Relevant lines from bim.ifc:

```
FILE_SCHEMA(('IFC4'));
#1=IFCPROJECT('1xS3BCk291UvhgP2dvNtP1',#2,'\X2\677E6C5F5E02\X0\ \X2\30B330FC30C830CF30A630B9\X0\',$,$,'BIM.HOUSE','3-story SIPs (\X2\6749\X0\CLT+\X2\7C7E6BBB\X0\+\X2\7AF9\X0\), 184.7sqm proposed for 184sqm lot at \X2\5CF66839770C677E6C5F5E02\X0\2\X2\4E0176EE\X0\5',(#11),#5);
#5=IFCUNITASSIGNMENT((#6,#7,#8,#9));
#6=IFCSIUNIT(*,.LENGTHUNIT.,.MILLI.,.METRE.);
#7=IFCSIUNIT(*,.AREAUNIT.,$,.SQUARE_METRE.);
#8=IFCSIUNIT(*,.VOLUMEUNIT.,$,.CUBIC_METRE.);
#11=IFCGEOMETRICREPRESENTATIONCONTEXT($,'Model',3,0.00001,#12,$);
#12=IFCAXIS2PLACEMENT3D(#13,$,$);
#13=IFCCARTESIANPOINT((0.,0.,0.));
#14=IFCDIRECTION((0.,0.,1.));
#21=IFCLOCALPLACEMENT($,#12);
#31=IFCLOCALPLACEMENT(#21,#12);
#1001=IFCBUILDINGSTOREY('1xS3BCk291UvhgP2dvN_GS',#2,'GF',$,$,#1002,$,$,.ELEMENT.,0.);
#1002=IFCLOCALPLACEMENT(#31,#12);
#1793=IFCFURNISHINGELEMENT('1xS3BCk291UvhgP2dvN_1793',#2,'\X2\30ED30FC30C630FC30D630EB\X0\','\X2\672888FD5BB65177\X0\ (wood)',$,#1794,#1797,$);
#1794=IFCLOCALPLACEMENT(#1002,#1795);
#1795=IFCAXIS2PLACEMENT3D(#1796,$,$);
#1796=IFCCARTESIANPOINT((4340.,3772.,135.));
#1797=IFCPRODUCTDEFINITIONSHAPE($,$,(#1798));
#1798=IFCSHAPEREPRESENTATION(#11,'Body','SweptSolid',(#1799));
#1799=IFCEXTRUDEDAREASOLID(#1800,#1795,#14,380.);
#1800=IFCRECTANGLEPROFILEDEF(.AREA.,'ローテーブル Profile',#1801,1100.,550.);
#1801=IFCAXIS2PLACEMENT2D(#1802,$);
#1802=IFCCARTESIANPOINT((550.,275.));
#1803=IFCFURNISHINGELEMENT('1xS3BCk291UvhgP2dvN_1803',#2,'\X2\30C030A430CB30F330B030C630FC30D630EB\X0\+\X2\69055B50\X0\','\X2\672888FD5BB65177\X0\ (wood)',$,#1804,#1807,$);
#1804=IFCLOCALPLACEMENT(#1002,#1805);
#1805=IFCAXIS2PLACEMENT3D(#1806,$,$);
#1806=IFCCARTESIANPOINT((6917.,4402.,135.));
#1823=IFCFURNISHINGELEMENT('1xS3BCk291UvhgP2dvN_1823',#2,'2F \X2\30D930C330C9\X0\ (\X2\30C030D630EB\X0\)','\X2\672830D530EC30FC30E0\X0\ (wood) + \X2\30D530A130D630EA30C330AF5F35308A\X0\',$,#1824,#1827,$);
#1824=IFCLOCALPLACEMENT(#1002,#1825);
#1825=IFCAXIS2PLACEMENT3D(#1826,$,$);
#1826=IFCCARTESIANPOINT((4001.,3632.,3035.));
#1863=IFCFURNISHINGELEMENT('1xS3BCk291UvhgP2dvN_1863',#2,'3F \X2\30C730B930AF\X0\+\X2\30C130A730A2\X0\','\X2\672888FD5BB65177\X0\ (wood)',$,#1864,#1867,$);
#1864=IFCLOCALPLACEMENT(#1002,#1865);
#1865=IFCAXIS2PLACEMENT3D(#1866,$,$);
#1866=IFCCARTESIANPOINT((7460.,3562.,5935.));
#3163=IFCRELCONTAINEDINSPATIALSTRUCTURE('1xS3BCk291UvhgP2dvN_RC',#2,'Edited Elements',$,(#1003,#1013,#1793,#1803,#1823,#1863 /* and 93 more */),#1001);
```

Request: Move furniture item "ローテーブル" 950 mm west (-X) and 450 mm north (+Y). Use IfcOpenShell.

```python
import ifcopenshell
import ifcopenshell.api.geometry
import ifcopenshell.util.placement
import ifcopenshell.util.unit

model = ifcopenshell.open("bim.ifc")
unit_scale = ifcopenshell.util.unit.calculate_unit_scale(model)

item = model.by_guid("1xS3BCk291UvhgP2dvN_1793")
matrix = ifcopenshell.util.placement.get_local_placement(item.ObjectPlacement)
matrix[0, 3] -= 0.95 / unit_scale
matrix[1, 3] += 0.45 / unit_scale
ifcopenshell.api.geometry.edit_object_placement(model, product=item, matrix=matrix, is_si=False)

print(ifcopenshell.util.placement.get_local_placement(item.ObjectPlacement).round(3) + 0.0)

model.write("bim_v2.ifc")
```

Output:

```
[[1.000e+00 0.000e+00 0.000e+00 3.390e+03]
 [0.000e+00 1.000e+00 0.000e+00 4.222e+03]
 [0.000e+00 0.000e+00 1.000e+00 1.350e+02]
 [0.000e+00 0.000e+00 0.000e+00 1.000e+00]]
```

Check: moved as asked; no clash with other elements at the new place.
